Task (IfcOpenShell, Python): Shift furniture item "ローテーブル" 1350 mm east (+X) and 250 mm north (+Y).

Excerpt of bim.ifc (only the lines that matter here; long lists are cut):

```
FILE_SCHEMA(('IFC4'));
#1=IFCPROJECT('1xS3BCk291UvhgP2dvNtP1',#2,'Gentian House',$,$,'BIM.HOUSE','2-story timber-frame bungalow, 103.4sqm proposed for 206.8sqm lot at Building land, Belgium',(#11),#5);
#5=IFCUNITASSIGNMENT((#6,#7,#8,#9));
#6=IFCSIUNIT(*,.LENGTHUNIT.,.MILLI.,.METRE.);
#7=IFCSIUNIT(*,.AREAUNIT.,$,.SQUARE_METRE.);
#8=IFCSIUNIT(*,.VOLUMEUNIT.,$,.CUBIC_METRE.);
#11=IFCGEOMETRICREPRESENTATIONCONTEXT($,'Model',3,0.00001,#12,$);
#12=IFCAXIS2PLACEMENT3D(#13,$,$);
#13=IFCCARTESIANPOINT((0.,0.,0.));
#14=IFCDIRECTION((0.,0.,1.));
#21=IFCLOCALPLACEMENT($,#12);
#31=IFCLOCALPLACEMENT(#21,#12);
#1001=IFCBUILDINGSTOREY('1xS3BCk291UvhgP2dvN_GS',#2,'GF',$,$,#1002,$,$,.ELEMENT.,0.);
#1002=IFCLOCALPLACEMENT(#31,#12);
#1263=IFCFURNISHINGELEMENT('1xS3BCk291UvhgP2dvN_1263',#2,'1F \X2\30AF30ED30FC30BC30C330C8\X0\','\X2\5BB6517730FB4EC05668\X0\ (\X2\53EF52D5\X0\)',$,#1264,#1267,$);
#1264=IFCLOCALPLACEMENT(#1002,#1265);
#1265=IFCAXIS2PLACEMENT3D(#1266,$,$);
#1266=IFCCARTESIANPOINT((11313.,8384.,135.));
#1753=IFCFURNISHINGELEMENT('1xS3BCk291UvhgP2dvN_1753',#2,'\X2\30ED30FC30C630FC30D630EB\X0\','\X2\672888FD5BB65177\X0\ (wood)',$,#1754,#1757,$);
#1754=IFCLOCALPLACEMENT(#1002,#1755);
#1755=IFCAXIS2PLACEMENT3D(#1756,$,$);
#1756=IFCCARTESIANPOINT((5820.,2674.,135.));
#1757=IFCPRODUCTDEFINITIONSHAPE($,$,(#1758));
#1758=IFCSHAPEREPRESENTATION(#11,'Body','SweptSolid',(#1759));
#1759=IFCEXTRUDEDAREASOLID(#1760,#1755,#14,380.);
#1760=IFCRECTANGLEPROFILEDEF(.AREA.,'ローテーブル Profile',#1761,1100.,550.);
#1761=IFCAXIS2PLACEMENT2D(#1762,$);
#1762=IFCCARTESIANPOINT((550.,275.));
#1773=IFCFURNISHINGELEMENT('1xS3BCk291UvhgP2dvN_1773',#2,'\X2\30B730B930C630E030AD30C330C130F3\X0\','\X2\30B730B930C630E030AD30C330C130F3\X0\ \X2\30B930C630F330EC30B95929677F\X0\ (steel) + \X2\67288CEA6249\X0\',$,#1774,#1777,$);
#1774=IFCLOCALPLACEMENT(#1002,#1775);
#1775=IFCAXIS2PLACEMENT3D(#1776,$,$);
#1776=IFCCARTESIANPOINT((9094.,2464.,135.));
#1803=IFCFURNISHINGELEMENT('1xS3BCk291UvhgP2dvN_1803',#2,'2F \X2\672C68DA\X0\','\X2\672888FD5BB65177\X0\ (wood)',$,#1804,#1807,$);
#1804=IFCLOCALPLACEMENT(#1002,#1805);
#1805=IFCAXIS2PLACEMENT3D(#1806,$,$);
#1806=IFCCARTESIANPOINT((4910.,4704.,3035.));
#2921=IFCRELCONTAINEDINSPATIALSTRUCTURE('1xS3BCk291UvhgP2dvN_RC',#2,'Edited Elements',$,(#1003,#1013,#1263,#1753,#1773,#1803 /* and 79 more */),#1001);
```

```python
import ifcopenshell
import ifcopenshell.api.geometry
import ifcopenshell.util.placement

model = ifcopenshell.open("bim.ifc")

item = model.by_guid("1xS3BCk291UvhgP2dvN_1753")
matrix = ifcopenshell.util.placement.get_local_placement(item.ObjectPlacement)
matrix[0, 3] += 1350.0
matrix[1, 3] += 250.0
ifcopenshell.api.geometry.edit_object_placement(model, product=item, matrix=matrix, is_si=False)

print(ifcopenshell.util.placement.get_local_placement(item.ObjectPlacement).round(3) + 0.0)

model.write("bim_edited.ifc")
```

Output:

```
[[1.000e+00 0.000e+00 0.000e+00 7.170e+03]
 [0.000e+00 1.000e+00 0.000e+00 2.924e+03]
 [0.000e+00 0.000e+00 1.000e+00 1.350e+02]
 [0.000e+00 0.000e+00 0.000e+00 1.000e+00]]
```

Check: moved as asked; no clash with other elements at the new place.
